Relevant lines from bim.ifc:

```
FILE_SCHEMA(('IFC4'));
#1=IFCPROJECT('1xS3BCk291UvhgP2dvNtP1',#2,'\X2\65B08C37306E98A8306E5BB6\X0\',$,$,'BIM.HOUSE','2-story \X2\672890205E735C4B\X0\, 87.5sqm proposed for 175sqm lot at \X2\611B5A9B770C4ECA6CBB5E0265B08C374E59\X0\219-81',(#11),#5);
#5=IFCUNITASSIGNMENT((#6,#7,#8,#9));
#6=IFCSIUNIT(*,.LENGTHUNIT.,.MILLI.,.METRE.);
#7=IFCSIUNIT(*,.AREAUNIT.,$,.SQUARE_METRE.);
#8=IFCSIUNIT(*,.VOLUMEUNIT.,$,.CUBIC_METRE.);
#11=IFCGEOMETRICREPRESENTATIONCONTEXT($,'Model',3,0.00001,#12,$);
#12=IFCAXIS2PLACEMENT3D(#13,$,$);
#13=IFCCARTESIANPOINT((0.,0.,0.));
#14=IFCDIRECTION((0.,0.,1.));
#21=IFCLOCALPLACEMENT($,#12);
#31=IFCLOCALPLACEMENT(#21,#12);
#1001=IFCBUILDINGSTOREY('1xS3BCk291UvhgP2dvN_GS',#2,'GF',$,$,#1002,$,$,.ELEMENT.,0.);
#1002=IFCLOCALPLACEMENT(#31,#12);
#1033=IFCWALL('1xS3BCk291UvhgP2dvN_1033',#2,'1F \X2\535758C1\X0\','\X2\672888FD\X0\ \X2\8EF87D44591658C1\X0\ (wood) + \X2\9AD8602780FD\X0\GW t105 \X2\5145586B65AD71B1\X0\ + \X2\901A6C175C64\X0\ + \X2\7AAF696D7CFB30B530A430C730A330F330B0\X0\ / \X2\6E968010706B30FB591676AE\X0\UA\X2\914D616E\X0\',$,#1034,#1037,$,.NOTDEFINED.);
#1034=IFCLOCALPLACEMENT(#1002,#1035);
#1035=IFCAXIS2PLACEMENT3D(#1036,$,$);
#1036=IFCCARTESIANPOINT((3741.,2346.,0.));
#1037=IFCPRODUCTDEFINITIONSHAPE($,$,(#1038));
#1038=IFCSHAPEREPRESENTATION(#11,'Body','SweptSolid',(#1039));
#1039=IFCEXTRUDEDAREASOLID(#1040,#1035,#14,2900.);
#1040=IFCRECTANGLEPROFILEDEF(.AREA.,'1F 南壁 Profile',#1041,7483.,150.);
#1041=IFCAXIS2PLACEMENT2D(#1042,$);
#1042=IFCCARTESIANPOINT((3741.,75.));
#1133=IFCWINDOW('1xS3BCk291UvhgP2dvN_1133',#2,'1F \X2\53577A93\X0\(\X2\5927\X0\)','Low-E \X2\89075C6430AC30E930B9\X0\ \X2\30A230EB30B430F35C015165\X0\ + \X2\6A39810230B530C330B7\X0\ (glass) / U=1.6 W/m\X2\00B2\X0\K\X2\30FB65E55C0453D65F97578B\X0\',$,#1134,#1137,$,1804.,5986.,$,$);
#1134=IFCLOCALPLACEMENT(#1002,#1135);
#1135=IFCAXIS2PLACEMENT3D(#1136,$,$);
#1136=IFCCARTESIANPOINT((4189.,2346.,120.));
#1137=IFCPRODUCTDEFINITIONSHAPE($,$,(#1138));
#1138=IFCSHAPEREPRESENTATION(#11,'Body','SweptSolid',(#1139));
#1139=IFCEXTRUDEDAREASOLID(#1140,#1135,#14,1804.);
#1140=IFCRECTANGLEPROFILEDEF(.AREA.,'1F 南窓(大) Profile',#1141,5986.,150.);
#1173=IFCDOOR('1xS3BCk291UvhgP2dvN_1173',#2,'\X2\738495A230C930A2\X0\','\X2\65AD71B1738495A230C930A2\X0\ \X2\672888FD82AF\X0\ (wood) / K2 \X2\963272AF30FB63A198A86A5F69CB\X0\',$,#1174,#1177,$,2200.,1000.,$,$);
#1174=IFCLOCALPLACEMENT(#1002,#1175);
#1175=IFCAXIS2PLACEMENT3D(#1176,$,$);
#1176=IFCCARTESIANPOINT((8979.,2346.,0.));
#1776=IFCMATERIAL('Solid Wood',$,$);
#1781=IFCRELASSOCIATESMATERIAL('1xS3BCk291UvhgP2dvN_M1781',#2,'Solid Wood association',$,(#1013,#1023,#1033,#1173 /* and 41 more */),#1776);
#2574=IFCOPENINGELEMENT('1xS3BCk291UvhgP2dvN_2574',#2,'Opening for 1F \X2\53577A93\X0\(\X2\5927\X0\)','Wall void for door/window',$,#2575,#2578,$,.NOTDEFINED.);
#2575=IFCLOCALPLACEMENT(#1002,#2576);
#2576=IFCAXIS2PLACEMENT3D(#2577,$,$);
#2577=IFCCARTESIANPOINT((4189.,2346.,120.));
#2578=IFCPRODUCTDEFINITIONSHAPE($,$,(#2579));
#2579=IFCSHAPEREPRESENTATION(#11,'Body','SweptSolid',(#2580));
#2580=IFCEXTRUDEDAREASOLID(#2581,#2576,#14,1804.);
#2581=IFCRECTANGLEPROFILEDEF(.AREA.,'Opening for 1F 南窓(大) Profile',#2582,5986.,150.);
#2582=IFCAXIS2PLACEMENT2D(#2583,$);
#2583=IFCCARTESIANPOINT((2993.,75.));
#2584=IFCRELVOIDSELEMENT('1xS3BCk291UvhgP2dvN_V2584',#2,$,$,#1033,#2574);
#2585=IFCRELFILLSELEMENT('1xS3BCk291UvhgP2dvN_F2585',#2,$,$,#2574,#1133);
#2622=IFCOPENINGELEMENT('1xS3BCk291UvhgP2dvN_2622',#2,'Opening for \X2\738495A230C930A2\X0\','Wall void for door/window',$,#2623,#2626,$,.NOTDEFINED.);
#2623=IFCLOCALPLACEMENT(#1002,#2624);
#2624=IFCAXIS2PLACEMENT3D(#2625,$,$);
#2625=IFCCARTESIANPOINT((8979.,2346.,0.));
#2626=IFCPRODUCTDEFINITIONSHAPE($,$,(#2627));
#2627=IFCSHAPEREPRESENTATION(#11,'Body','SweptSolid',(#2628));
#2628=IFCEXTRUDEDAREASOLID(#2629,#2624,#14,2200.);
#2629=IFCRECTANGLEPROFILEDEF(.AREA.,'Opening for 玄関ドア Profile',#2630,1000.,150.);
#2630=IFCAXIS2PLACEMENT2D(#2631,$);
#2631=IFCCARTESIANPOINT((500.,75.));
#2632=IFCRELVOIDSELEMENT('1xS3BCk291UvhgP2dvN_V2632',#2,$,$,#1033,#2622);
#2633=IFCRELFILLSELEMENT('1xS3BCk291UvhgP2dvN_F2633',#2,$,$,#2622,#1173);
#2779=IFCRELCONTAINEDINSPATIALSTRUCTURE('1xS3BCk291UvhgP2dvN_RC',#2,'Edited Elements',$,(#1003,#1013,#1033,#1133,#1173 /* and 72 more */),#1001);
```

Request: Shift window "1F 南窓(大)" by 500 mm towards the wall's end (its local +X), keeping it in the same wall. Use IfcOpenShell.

```python
import ifcopenshell
import ifcopenshell.api.geometry
import ifcopenshell.util.placement
import ifcopenshell.util.unit

model = ifcopenshell.open("bim.ifc")
unit_scale = ifcopenshell.util.unit.calculate_unit_scale(model)

window = model.by_guid("1xS3BCk291UvhgP2dvN_1133")
opening = window.FillsVoids[0].RelatingOpeningElement
wall = opening.VoidsElements[0].RelatingBuildingElement

wall_matrix = ifcopenshell.util.placement.get_local_placement(wall.ObjectPlacement)
shift = wall_matrix[:3, 0] * 0.5 / unit_scale
before = ifcopenshell.util.placement.get_local_placement(window.ObjectPlacement)[:3, 3].copy()

# The window is not placed relative to its opening, so move both.
for product in (opening, window):
    matrix = ifcopenshell.util.placement.get_local_placement(product.ObjectPlacement)
    matrix[:3, 3] += shift
    ifcopenshell.api.geometry.edit_object_placement(model, product=product, matrix=matrix, is_si=False)

after = ifcopenshell.util.placement.get_local_placement(window.ObjectPlacement)[:3, 3]
print("window moved by", (after - before).round(3) + 0.0)

model.write("bim_rev.ifc")
```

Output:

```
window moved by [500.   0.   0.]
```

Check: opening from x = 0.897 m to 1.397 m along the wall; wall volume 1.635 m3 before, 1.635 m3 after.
